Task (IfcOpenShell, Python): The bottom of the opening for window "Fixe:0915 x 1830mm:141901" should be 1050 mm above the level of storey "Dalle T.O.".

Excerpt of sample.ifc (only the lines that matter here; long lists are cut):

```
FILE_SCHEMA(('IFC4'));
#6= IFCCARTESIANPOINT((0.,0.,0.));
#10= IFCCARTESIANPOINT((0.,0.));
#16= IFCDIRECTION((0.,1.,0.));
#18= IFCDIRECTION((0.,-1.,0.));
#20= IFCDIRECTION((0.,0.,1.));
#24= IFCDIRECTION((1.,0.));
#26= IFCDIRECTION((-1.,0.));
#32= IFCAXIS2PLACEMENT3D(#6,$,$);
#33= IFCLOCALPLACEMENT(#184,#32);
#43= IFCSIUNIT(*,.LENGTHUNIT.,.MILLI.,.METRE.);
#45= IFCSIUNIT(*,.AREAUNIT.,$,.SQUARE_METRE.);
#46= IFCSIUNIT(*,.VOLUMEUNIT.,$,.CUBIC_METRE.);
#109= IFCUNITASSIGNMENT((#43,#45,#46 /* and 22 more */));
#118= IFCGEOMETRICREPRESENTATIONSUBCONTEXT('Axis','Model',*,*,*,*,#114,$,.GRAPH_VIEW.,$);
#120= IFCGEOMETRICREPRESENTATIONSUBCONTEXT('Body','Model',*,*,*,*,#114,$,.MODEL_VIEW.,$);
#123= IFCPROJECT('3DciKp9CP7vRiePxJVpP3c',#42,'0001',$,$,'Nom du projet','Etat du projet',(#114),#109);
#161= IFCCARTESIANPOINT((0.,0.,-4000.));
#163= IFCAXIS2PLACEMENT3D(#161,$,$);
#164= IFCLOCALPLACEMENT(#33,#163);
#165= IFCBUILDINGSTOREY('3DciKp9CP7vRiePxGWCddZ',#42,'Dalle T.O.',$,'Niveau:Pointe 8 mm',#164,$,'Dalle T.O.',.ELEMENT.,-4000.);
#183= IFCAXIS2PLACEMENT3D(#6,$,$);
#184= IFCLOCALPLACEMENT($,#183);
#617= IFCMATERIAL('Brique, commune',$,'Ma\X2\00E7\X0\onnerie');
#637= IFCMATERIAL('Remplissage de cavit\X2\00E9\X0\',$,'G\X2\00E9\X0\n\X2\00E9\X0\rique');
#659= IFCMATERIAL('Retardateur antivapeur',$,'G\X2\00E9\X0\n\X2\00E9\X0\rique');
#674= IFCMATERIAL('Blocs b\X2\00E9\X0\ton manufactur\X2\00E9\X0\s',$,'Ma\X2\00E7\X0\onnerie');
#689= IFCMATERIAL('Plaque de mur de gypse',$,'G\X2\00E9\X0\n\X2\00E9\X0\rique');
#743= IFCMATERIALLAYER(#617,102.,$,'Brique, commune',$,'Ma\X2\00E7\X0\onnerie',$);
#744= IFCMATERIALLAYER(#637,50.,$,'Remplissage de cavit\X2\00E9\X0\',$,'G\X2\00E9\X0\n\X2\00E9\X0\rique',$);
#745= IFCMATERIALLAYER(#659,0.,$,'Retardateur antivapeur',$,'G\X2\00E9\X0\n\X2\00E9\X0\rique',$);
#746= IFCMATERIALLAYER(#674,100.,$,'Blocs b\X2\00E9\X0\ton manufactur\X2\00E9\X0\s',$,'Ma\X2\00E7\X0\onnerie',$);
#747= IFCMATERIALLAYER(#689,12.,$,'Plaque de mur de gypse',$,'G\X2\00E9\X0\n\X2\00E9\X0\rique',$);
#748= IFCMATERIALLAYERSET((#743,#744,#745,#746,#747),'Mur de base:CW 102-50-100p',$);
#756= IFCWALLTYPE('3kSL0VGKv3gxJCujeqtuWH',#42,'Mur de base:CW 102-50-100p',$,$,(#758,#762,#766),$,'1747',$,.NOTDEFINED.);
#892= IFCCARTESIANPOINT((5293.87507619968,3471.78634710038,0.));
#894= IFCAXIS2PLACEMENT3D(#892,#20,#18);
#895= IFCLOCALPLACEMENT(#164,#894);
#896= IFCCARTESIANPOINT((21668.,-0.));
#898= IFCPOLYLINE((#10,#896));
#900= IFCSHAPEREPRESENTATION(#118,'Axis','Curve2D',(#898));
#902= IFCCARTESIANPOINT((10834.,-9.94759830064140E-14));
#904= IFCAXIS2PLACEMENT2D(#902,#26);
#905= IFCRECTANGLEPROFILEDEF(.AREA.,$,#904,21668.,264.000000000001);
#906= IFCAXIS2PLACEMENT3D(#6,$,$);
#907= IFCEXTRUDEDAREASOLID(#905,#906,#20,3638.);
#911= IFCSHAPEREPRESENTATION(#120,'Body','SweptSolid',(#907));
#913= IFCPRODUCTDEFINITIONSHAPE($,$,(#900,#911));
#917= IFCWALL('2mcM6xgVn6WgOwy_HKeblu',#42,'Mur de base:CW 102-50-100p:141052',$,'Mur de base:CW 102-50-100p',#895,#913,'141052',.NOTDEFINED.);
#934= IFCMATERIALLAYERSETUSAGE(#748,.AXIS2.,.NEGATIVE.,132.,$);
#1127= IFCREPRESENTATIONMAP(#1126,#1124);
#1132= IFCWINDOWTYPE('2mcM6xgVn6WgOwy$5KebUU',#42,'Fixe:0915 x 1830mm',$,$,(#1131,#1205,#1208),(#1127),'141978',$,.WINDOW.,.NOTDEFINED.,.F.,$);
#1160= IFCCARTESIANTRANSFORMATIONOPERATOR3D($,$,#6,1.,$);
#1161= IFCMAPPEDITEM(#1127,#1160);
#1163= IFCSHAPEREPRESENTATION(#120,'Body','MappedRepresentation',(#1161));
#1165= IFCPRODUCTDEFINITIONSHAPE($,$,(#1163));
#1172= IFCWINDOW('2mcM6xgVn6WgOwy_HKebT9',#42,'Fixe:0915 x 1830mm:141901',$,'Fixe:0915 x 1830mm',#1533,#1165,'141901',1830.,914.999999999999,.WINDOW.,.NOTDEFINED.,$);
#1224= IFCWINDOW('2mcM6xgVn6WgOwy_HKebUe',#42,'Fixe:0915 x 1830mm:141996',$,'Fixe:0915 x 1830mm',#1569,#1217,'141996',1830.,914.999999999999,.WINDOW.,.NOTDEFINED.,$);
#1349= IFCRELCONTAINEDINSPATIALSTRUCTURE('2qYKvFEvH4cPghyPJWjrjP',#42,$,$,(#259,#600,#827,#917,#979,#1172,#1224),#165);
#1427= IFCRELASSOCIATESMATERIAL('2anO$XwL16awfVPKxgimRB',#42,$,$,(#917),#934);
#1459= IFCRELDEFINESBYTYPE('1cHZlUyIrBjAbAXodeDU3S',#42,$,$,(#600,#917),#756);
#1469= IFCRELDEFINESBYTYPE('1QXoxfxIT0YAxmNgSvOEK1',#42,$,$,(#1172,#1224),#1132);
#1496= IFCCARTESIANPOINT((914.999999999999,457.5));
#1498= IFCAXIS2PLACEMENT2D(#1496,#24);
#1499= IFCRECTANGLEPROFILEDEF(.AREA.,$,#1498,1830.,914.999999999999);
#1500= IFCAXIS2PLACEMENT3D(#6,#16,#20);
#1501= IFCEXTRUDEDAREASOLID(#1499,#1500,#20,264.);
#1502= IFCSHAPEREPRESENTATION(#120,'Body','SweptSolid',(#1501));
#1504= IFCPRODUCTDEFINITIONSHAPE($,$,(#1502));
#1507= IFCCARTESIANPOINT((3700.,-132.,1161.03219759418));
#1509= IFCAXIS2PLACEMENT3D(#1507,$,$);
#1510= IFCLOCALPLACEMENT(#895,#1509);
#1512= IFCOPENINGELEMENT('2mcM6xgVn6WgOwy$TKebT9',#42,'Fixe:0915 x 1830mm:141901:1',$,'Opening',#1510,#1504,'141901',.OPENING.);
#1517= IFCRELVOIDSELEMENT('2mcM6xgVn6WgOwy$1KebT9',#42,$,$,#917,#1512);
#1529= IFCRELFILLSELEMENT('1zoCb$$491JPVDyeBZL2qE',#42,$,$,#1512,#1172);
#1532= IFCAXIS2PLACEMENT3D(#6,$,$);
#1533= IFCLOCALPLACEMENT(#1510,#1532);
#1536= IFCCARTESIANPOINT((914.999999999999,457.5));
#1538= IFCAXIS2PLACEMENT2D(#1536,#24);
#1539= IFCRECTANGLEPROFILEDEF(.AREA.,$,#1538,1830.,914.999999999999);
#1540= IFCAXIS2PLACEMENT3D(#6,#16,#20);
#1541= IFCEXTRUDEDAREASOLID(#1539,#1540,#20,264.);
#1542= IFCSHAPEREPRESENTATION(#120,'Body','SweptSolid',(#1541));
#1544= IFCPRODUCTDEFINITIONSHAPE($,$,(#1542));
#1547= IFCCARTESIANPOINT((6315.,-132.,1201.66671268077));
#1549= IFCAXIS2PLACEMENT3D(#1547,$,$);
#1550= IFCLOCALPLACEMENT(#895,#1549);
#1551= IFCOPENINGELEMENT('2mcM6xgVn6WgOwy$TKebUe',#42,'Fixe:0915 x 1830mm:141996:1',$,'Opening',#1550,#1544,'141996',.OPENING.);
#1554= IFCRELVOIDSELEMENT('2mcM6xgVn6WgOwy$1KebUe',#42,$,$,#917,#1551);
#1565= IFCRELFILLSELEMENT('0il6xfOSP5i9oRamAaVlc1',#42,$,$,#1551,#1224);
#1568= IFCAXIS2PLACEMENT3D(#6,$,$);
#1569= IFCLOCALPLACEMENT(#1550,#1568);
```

```python
import numpy as np
import ifcopenshell
import ifcopenshell.api.geometry
import ifcopenshell.geom
import ifcopenshell.util.element
import ifcopenshell.util.placement
import ifcopenshell.util.shape
import ifcopenshell.util.unit

model = ifcopenshell.open("sample.ifc")
unit_scale = ifcopenshell.util.unit.calculate_unit_scale(model)

window = model.by_guid("2mcM6xgVn6WgOwy_HKebT9")
opening = window.FillsVoids[0].RelatingOpeningElement
storey = ifcopenshell.util.element.get_container(window, ifc_class="IfcBuildingStorey")
level = ifcopenshell.util.placement.get_local_placement(storey.ObjectPlacement)[2, 3]

# The opening's origin need not be at the sill, so measure its lowest point.
shape = ifcopenshell.geom.create_shape(ifcopenshell.geom.settings(), opening)
bottom = ifcopenshell.util.shape.get_shape_bottom_elevation(shape, shape.geometry) / unit_scale
dz = level + 1.05 / unit_scale - bottom

shift = np.array([0.0, 0.0, dz])
# The window is placed relative to its opening, so it follows when the opening moves.
matrix = ifcopenshell.util.placement.get_local_placement(opening.ObjectPlacement)
matrix[:3, 3] += shift
ifcopenshell.api.geometry.edit_object_placement(
    model, product=opening, matrix=matrix, is_si=False, should_transform_children=True
)

print(f"moved by {dz * unit_scale:+.3f} m")

model.write("sample_updated.ifc")
```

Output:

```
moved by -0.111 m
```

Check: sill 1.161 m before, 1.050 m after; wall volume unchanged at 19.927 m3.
